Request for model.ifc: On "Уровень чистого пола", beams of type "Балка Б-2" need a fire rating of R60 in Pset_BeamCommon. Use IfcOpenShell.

First a look at what the model holds.

```python
import ifcopenshell
import ifcopenshell.util.element

model = ifcopenshell.open("model.ifc")
print(model.schema)
storey = next(s for s in model.by_type("IfcBuildingStorey") if s.Name == "Уровень чистого пола")
beams = [e for e in ifcopenshell.util.element.get_decomposition(storey) if e.is_a("IfcBeam")]
seen = {}
for e in beams:
    element_type = ifcopenshell.util.element.get_type(e)
    key = (element_type.Name if element_type != e and element_type else None, ifcopenshell.util.element.get_pset(e, "Pset_BeamCommon", "FireRating"))
    seen[key] = seen.get(key, 0) + 1
for (name, value), count in sorted(seen.items(), key=str):
    print(count, "x", name, "|", value)
```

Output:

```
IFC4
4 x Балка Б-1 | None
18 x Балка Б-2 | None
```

```python
import ifcopenshell
import ifcopenshell.api.pset
import ifcopenshell.util.element

model = ifcopenshell.open("model.ifc")

storey = next(s for s in model.by_type("IfcBuildingStorey") if s.Name == "Уровень чистого пола")
beams = [e for e in ifcopenshell.util.element.get_decomposition(storey) if e.is_a("IfcBeam")]

count = 0
for e in beams:
    element_type = ifcopenshell.util.element.get_type(e)
    if element_type in (None, e) or element_type.Name != "Балка Б-2":
        continue
    # add_pset returns the element's existing set when there is one.
    pset = ifcopenshell.api.pset.add_pset(model, product=e, name="Pset_BeamCommon")
    ifcopenshell.api.pset.edit_pset(model, pset=pset, properties={"FireRating": "R60"})
    count += 1

print(count, "beams updated")

model.write("model_rev.ifc")
```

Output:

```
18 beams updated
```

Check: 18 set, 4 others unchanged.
